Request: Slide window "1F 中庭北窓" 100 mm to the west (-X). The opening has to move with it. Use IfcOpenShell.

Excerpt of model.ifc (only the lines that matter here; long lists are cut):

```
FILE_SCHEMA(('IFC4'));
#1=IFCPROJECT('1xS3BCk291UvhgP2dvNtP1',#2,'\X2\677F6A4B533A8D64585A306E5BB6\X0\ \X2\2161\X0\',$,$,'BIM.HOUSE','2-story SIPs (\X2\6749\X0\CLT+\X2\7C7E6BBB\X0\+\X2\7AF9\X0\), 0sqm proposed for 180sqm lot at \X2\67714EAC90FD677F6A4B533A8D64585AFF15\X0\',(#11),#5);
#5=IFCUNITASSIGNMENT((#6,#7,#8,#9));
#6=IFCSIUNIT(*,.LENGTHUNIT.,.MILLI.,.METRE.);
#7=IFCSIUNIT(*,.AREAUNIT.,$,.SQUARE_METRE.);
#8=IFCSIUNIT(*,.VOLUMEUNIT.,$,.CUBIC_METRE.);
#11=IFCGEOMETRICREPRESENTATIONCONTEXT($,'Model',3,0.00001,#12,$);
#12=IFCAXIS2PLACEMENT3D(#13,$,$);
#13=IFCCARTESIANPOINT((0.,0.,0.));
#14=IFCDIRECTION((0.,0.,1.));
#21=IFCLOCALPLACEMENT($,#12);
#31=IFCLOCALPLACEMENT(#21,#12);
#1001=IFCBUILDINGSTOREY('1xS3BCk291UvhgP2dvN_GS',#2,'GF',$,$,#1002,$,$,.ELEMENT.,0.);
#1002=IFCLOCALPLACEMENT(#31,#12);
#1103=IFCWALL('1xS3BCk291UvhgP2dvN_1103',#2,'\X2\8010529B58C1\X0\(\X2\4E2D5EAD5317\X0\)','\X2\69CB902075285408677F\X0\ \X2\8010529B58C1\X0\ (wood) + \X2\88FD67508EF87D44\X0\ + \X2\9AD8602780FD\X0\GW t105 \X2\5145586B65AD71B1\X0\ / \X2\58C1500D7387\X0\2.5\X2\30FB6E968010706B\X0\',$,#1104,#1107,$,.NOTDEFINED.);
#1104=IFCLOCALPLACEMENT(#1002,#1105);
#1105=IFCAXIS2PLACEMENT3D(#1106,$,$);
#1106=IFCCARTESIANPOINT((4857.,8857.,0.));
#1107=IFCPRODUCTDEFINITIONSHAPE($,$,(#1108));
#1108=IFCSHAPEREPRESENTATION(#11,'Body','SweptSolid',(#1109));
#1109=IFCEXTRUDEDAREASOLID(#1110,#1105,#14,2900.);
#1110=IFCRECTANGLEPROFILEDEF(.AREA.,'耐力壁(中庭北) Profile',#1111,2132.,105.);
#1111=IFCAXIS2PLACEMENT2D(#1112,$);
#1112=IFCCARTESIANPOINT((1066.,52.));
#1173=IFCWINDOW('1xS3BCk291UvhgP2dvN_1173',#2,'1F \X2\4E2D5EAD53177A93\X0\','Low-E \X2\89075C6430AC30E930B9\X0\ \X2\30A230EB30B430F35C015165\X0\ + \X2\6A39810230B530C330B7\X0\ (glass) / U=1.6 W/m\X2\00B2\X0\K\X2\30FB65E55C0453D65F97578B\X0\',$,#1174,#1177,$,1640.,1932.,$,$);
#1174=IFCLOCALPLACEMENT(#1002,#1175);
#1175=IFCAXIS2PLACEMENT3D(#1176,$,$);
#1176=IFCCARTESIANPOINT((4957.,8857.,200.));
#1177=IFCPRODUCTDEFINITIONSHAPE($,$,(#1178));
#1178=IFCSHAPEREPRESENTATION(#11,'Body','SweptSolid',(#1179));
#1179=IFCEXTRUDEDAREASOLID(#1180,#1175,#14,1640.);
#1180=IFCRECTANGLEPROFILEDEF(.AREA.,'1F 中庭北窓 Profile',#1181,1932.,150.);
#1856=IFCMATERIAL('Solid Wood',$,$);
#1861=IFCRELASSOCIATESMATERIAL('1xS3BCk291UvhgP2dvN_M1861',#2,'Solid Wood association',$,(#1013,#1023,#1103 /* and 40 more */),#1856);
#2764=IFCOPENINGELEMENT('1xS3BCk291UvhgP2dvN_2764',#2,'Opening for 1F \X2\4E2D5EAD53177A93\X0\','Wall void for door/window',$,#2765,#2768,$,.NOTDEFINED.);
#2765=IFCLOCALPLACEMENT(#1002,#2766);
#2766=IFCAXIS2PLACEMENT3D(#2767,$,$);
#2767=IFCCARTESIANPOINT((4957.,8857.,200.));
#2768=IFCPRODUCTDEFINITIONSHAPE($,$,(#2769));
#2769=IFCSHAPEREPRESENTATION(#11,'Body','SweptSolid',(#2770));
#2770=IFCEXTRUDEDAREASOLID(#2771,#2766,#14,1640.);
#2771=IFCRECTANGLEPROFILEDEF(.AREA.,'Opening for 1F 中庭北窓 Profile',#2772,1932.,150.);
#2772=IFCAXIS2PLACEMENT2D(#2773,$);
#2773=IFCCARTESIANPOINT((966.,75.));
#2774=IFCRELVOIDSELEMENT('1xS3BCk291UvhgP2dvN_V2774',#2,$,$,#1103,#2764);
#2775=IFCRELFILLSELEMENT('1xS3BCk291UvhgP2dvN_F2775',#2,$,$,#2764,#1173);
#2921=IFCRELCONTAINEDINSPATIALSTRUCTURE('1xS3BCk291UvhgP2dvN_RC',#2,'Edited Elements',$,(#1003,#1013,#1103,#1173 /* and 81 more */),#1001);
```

```python
import ifcopenshell
import ifcopenshell.api.geometry
import ifcopenshell.util.placement
import ifcopenshell.util.unit

model = ifcopenshell.open("model.ifc")
unit_scale = ifcopenshell.util.unit.calculate_unit_scale(model)

window = model.by_id(1173)
opening = window.FillsVoids[0].RelatingOpeningElement
wall = opening.VoidsElements[0].RelatingBuildingElement

wall_matrix = ifcopenshell.util.placement.get_local_placement(wall.ObjectPlacement)
shift = wall_matrix[:3, 0] * -0.1 / unit_scale
before = ifcopenshell.util.placement.get_local_placement(window.ObjectPlacement)[:3, 3].copy()

# The window is not placed relative to its opening, so move both.
for product in (opening, window):
    matrix = ifcopenshell.util.placement.get_local_placement(product.ObjectPlacement)
    matrix[:3, 3] += shift
    ifcopenshell.api.geometry.edit_object_placement(model, product=product, matrix=matrix, is_si=False)

after = ifcopenshell.util.placement.get_local_placement(window.ObjectPlacement)[:3, 3]
print("window moved by", (after - before).round(3) + 0.0)

model.write("model_edited.ifc")
```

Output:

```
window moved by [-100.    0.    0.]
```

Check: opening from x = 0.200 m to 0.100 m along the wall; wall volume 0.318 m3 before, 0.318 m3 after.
